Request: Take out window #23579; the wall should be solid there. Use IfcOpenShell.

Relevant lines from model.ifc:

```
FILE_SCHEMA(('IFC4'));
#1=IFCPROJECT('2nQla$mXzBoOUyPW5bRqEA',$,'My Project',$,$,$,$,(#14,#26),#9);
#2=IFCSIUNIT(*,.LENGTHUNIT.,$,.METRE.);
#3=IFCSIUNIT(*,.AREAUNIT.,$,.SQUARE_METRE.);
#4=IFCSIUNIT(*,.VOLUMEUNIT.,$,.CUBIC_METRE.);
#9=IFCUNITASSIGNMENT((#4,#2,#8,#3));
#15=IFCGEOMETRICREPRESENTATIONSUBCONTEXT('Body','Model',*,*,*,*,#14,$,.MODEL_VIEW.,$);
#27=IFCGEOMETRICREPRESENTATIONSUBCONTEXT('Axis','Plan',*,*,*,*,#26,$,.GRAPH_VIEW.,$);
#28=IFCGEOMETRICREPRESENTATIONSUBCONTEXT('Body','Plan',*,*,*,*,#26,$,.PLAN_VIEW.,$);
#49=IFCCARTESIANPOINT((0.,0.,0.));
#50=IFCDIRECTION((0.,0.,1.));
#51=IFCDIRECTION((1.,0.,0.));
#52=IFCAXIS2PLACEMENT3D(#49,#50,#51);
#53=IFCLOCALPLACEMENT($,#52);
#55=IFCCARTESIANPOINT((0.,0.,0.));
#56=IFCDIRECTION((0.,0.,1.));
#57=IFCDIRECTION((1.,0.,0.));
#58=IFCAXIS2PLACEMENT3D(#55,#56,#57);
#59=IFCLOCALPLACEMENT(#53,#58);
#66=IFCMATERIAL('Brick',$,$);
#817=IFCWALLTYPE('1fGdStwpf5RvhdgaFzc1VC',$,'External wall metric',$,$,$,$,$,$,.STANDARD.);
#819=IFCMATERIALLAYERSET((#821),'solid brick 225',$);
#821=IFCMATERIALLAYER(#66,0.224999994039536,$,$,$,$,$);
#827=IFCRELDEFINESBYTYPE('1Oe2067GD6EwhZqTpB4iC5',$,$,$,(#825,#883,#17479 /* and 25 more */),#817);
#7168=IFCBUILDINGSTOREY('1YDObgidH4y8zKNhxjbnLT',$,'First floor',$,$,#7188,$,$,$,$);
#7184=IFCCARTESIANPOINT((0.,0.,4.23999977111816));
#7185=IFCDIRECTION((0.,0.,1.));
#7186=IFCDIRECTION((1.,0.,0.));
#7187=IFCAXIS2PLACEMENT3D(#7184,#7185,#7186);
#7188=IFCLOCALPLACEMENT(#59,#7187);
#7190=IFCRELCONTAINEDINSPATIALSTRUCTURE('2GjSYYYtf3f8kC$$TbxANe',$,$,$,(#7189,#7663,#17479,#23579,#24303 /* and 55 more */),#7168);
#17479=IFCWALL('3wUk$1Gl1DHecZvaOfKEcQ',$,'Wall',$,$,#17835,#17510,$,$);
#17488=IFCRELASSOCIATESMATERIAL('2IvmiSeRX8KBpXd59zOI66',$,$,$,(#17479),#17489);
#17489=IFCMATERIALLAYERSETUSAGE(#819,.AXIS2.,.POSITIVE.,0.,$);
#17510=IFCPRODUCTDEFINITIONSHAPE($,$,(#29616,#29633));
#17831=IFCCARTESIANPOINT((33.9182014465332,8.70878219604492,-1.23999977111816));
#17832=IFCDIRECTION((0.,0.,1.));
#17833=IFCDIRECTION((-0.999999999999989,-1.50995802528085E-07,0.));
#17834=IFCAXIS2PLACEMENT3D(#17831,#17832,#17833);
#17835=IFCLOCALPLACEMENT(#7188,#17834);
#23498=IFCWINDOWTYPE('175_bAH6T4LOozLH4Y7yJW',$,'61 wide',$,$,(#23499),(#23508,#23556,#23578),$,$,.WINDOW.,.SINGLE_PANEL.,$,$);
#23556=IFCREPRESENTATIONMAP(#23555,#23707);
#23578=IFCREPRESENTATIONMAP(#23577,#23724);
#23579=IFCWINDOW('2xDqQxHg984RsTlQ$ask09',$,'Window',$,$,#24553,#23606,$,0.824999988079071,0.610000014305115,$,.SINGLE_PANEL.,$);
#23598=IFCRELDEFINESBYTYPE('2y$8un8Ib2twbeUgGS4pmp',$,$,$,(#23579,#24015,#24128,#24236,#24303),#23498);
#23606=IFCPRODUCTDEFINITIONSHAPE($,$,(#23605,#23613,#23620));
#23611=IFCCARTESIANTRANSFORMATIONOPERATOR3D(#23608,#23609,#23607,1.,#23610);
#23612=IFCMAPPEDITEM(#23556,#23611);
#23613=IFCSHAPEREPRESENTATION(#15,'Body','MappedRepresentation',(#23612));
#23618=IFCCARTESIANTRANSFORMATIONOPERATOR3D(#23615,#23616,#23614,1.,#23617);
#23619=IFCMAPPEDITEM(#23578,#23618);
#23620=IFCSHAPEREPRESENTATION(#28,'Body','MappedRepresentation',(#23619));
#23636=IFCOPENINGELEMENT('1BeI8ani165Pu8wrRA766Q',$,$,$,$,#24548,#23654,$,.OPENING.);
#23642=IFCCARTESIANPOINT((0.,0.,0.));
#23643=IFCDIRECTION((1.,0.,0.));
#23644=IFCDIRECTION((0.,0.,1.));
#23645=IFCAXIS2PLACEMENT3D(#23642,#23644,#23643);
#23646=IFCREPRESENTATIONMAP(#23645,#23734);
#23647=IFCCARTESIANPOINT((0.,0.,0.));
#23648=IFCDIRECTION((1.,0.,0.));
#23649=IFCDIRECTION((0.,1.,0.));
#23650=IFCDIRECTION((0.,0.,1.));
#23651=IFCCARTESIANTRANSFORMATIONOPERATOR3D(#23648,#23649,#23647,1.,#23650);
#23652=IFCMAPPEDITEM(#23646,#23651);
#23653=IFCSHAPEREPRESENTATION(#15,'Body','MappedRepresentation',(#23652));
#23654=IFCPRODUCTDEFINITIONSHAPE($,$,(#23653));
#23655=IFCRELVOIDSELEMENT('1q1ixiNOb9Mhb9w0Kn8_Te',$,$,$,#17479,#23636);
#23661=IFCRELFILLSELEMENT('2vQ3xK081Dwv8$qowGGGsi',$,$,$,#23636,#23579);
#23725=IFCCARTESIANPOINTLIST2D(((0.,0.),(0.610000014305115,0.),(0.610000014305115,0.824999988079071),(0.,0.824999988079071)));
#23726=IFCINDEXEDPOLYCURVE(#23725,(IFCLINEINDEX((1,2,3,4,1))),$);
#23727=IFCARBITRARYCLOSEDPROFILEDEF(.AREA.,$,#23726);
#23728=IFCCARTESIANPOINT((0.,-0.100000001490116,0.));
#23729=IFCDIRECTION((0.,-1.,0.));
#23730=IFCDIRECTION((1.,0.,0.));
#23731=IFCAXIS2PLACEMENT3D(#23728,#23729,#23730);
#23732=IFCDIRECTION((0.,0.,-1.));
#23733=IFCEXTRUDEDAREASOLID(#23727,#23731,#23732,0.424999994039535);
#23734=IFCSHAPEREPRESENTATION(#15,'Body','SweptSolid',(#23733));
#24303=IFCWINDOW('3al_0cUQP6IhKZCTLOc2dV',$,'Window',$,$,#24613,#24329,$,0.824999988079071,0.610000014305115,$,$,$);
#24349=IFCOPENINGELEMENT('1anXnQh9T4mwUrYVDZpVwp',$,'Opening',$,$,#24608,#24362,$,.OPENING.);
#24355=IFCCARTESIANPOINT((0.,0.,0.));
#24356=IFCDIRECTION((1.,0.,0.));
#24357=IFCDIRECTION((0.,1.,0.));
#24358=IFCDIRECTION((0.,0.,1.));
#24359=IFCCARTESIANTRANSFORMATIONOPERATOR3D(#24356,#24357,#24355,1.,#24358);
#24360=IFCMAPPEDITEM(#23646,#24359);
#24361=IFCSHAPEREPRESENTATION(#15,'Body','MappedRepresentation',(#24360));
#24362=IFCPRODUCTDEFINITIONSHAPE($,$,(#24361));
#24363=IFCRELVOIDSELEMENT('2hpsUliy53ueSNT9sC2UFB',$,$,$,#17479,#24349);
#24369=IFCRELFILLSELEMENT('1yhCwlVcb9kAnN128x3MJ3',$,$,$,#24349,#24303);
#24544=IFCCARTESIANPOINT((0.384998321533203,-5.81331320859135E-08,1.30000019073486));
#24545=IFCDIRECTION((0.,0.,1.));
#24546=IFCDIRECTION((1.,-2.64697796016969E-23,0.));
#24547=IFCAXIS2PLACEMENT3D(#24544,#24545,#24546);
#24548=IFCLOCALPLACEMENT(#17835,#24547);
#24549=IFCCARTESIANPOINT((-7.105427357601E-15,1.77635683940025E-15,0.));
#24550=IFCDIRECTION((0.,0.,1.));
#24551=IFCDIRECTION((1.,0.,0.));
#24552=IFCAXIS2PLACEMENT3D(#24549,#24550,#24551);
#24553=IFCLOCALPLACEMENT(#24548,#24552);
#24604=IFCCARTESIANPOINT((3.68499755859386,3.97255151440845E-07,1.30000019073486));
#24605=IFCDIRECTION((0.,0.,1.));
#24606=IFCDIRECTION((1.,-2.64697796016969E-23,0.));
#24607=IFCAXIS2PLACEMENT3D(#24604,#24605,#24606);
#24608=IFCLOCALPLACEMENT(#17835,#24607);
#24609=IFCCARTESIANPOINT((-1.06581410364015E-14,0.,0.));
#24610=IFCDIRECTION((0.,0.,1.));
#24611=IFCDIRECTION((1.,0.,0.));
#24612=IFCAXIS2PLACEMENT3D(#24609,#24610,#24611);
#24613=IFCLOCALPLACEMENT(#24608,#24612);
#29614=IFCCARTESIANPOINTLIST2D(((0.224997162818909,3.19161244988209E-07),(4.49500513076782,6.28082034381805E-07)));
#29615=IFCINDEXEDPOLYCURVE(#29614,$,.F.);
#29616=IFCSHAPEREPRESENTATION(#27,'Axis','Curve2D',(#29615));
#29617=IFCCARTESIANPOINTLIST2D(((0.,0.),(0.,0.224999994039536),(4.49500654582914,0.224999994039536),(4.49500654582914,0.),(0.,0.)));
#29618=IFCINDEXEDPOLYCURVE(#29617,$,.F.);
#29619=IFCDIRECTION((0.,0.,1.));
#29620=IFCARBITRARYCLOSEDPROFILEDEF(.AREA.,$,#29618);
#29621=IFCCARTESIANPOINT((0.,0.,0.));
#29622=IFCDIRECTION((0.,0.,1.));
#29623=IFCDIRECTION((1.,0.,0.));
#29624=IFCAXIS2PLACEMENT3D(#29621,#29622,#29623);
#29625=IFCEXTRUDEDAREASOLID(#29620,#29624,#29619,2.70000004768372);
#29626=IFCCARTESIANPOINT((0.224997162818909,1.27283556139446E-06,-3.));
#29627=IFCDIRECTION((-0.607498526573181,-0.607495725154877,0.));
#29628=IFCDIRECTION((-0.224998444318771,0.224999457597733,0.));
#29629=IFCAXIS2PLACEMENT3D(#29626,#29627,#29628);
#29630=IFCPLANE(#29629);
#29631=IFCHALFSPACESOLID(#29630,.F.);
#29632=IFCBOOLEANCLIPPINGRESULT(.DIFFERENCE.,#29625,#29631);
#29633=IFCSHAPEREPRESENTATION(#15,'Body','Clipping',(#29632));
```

```python
import ifcopenshell
import ifcopenshell.api.feature
import ifcopenshell.api.root
import ifcopenshell.geom
import ifcopenshell.util.shape

model = ifcopenshell.open("model.ifc")
settings = ifcopenshell.geom.settings()


def volume(element):
    """Net volume in cubic metres, openings subtracted."""
    shape = ifcopenshell.geom.create_shape(settings, element)
    return ifcopenshell.util.shape.get_volume(shape.geometry)


window = model.by_id(23579)
opening = window.FillsVoids[0].RelatingOpeningElement
wall = opening.VoidsElements[0].RelatingBuildingElement
before = volume(wall)

ifcopenshell.api.root.remove_product(model, product=window)
ifcopenshell.api.feature.remove_feature(model, feature=opening)

after = volume(wall)

print(f"wall volume {before:.3f} -> {after:.3f} m3")

model.write("model_rev.ifc")
```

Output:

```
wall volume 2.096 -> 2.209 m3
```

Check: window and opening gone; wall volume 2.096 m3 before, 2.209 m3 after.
